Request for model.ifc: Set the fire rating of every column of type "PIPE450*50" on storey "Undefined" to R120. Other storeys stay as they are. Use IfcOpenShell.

First a look at what the model holds.

```python
import ifcopenshell
import ifcopenshell.util.element

model = ifcopenshell.open("model.ifc")
print(model.schema)
storey = next(s for s in model.by_type("IfcBuildingStorey") if s.Name == "Undefined")
columns = [e for e in ifcopenshell.util.element.get_decomposition(storey) if e.is_a("IfcColumn")]
seen = {}
for e in columns:
    element_type = ifcopenshell.util.element.get_type(e)
    key = (element_type.Name if element_type != e and element_type else None, ifcopenshell.util.element.get_pset(e, "Pset_ColumnCommon", "FireRating"))
    seen[key] = seen.get(key, 0) + 1
for (name, value), count in sorted(seen.items(), key=str):
    print(count, "x", name, "|", value)
```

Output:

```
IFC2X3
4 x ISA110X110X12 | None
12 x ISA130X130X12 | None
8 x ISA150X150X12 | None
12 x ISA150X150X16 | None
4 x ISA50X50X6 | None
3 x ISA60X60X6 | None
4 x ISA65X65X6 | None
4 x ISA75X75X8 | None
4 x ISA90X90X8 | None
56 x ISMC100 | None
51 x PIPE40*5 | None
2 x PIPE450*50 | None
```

```python
import ifcopenshell
import ifcopenshell.api.pset
import ifcopenshell.util.element

model = ifcopenshell.open("model.ifc")

storey = next(s for s in model.by_type("IfcBuildingStorey") if s.Name == "Undefined")
columns = [e for e in ifcopenshell.util.element.get_decomposition(storey) if e.is_a("IfcColumn")]

count = 0
for e in columns:
    element_type = ifcopenshell.util.element.get_type(e)
    if element_type in (None, e) or element_type.Name != "PIPE450*50":
        continue
    found = ifcopenshell.util.element.get_pset(e, "Pset_ColumnCommon", should_inherit=False)
    if found:
        pset = model.by_id(found["id"])
        if len(ifcopenshell.util.element.get_elements_by_pset(pset)) > 1:
            pset = ifcopenshell.api.pset.unshare_pset(model, products=[e], pset=pset)[0]
    else:
        pset = ifcopenshell.api.pset.add_pset(model, product=e, name="Pset_ColumnCommon")
    ifcopenshell.api.pset.edit_pset(model, pset=pset, properties={"FireRating": "R120"})
    count += 1

print(count, "columns updated")

model.write("model_edited.ifc")
```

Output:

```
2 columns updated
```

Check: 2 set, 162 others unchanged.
